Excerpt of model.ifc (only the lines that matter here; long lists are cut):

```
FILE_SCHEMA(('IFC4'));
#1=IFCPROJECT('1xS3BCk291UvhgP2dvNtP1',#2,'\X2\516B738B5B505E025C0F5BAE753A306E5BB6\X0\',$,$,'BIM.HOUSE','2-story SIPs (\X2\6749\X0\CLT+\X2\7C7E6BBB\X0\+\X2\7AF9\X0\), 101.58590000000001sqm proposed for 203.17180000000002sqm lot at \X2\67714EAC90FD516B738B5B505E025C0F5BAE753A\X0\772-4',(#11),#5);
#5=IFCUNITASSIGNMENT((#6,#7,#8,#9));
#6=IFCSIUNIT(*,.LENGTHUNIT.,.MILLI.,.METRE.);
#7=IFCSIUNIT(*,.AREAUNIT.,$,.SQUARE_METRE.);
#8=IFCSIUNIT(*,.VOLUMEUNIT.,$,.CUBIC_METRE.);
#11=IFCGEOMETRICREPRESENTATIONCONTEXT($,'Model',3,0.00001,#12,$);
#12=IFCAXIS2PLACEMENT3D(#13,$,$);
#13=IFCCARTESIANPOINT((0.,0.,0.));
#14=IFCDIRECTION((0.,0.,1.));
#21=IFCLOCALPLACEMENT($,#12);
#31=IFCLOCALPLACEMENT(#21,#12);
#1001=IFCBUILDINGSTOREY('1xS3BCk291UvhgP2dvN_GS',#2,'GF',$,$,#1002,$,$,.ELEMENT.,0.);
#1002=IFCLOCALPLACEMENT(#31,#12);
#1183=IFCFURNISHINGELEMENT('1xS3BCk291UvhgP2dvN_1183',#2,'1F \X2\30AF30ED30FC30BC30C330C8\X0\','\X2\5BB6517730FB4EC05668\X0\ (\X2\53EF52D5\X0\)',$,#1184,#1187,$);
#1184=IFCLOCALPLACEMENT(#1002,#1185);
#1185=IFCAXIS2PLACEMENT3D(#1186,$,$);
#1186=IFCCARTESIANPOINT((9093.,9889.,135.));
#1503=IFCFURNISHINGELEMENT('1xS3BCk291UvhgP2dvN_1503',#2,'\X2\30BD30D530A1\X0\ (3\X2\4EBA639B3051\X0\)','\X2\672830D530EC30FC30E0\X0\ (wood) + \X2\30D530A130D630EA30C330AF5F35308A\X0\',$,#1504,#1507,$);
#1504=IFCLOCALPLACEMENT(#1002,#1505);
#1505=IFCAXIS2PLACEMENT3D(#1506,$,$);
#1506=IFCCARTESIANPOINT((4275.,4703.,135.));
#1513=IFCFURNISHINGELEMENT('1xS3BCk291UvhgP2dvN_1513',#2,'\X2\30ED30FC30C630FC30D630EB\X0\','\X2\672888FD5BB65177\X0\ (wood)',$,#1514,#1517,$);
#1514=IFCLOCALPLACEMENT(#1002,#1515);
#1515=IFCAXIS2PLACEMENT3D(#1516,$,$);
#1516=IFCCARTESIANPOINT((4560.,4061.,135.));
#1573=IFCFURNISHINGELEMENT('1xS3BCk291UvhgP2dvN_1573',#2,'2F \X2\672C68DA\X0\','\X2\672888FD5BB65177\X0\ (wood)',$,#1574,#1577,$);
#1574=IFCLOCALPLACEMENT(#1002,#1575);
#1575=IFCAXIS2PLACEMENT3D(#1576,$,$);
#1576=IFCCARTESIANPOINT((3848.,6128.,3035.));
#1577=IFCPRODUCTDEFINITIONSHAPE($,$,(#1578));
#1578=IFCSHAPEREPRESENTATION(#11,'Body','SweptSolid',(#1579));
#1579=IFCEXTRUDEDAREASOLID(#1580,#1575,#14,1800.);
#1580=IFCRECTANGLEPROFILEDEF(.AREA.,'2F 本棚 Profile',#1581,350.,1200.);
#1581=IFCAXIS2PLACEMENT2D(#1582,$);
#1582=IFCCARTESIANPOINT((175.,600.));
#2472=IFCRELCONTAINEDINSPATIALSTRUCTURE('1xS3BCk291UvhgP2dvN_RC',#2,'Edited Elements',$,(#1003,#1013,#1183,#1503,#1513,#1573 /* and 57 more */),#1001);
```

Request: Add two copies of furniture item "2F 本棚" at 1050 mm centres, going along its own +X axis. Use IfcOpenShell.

```python
import ifcopenshell
import ifcopenshell.api.geometry
import ifcopenshell.api.root
import ifcopenshell.util.element
import ifcopenshell.util.placement
import ifcopenshell.util.unit

model = ifcopenshell.open("model.ifc")
unit_scale = ifcopenshell.util.unit.calculate_unit_scale(model)


def reuse_history(source, copy):
    """copy_class also copies each property set's owner history, people and application; keep the originals."""
    for rel in copy.IsDefinedBy:
        if rel.is_a("IfcRelDefinesByProperties") and (history := rel.RelatingPropertyDefinition.OwnerHistory):
            rel.RelatingPropertyDefinition.OwnerHistory = source.OwnerHistory
            ifcopenshell.util.element.remove_deep2(model, history)


source = model.by_id(1573)
base = ifcopenshell.util.placement.get_local_placement(source.ObjectPlacement)
step = base[:3, 0] * 1.05 / unit_scale

for i in range(1, 3):
    copy = ifcopenshell.api.root.copy_class(model, product=source)
    copy.Representation = ifcopenshell.util.element.copy_deep(
        model, source.Representation, exclude=["IfcGeometricRepresentationContext", "IfcRepresentationMap"]
    )
    reuse_history(source, copy)
    matrix = base.copy()
    matrix[:3, 3] += i * step
    print("added at", matrix[:3, 3].round(3) + 0.0)
    ifcopenshell.api.geometry.edit_object_placement(model, product=copy, matrix=matrix, is_si=False)

model.write("model_updated.ifc")
```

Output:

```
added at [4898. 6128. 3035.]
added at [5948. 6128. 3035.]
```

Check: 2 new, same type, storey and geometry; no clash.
